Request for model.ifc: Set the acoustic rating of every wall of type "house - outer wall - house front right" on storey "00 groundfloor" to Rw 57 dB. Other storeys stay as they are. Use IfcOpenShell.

First a look at what the model holds.

```python
import ifcopenshell
import ifcopenshell.util.element

model = ifcopenshell.open("model.ifc")
print(model.schema)
storey = next(s for s in model.by_type("IfcBuildingStorey") if s.Name == "00 groundfloor")
walls = [e for e in ifcopenshell.util.element.get_decomposition(storey) if e.is_a("IfcWall")]
seen = {}
for e in walls:
    element_type = ifcopenshell.util.element.get_type(e)
    key = (element_type.Name if element_type != e and element_type else None, ifcopenshell.util.element.get_pset(e, "Pset_WallCommon", "AcousticRating"))
    seen[key] = seen.get(key, 0) + 1
for (name, value), count in sorted(seen.items(), key=str):
    print(count, "x", name, "|", value)
```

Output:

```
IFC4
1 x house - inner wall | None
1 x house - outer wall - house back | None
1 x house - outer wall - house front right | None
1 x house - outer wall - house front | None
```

```python
import ifcopenshell
import ifcopenshell.api.pset
import ifcopenshell.util.element

model = ifcopenshell.open("model.ifc")

storey = next(s for s in model.by_type("IfcBuildingStorey") if s.Name == "00 groundfloor")
walls = [e for e in ifcopenshell.util.element.get_decomposition(storey) if e.is_a("IfcWall")]

count = 0
for e in walls:
    element_type = ifcopenshell.util.element.get_type(e)
    if element_type in (None, e) or element_type.Name != "house - outer wall - house front right":
        continue
    # add_pset returns the element's existing set when there is one.
    pset = ifcopenshell.api.pset.add_pset(model, product=e, name="Pset_WallCommon")
    ifcopenshell.api.pset.edit_pset(model, pset=pset, properties={"AcousticRating": "Rw 57 dB"})
    count += 1

print(count, "walls updated")

model.write("model_edited.ifc")
```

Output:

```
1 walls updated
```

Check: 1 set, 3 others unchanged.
